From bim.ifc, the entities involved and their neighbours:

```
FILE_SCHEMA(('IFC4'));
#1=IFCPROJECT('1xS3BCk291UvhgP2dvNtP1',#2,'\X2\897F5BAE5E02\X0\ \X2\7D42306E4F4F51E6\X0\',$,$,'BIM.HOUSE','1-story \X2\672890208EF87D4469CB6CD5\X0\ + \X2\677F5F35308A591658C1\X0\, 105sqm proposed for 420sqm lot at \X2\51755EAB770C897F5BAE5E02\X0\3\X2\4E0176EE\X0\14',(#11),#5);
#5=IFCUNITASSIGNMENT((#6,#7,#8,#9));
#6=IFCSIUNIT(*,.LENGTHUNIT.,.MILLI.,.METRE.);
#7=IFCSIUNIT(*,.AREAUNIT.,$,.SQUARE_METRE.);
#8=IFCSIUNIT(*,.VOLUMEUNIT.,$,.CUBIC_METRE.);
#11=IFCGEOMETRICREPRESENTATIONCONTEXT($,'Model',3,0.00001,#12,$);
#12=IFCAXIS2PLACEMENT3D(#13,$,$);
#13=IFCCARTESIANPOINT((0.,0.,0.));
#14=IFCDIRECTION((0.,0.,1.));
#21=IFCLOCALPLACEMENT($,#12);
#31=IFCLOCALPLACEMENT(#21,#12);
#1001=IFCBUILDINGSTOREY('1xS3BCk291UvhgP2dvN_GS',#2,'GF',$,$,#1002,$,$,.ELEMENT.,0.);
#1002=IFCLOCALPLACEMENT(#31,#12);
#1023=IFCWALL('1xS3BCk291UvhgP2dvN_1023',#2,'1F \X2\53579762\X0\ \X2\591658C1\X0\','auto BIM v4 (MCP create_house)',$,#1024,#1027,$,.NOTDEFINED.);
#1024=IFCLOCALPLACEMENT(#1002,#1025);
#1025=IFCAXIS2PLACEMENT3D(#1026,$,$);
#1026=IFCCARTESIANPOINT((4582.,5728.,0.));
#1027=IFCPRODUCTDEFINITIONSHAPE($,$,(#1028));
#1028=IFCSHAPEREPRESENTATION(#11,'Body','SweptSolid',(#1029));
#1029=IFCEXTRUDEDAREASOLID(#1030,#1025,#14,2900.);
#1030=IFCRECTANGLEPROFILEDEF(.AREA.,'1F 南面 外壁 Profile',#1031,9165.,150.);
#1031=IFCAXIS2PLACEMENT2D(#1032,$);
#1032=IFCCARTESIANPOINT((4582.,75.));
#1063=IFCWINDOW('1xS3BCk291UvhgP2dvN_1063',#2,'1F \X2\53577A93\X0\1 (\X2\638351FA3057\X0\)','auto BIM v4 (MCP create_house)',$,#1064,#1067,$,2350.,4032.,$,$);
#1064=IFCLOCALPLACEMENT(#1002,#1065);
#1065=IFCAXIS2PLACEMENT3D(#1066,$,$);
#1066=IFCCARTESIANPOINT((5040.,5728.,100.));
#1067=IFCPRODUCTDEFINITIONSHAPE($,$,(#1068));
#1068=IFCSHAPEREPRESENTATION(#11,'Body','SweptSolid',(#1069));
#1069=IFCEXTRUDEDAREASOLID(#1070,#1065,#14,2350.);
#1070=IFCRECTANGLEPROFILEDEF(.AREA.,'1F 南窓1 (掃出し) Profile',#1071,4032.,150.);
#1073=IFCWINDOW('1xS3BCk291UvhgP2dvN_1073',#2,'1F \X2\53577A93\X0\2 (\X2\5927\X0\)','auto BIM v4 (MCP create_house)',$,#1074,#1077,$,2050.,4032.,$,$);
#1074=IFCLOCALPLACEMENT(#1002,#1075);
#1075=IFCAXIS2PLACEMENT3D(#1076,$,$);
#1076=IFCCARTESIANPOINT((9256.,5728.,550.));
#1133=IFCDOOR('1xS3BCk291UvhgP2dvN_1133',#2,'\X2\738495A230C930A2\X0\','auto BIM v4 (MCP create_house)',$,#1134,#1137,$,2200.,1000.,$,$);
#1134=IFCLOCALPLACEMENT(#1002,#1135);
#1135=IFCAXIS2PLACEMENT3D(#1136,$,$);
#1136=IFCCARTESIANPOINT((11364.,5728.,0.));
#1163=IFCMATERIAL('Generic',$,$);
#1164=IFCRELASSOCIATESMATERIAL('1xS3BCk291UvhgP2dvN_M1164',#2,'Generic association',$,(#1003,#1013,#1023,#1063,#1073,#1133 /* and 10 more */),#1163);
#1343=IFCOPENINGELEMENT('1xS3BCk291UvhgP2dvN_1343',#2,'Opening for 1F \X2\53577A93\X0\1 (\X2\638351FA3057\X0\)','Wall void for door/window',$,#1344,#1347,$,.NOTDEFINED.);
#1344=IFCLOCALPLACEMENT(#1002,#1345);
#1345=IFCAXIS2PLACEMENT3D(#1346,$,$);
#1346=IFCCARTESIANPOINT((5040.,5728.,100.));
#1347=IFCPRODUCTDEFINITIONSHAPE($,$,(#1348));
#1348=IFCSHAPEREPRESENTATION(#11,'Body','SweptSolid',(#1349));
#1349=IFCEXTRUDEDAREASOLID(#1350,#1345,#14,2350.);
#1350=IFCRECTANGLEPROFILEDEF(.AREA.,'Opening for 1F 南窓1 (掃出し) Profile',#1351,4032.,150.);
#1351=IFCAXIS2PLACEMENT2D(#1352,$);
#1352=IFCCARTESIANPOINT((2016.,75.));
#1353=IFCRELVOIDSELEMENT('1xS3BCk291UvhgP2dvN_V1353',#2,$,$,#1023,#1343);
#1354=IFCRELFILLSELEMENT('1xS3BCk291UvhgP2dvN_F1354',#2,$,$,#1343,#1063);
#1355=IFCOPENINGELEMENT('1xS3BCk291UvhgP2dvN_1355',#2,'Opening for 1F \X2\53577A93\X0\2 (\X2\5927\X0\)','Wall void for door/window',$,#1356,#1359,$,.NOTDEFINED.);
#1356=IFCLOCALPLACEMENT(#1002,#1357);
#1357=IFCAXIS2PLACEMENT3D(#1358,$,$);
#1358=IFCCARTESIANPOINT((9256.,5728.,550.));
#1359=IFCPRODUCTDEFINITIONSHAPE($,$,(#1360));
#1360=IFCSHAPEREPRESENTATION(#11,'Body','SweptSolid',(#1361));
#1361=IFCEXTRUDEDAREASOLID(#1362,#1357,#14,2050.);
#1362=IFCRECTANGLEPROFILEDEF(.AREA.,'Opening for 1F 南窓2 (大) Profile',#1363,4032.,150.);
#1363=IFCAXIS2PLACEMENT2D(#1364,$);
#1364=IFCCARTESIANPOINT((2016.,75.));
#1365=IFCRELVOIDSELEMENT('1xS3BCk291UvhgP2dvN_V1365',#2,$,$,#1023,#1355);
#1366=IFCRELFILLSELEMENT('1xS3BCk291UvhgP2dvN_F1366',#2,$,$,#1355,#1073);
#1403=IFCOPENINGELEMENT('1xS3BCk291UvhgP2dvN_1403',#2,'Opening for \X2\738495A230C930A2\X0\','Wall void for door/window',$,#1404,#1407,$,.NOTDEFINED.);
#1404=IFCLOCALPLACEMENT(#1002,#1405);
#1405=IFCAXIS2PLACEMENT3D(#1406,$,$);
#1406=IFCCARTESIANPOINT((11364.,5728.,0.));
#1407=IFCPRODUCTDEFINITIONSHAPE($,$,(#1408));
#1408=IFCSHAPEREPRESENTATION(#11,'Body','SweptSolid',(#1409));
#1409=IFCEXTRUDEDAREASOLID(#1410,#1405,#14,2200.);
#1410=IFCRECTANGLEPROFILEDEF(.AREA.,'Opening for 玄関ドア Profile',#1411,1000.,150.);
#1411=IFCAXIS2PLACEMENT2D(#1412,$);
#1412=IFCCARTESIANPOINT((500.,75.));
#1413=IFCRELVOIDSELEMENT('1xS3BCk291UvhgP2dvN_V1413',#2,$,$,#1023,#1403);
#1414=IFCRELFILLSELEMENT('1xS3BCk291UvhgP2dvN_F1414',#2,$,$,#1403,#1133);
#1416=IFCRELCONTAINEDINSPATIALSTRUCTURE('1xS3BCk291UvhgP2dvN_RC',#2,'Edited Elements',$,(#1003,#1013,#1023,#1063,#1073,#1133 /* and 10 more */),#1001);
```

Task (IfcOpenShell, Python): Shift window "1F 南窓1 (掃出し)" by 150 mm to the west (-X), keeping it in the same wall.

```python
import ifcopenshell
import ifcopenshell.api.geometry
import ifcopenshell.util.placement
import ifcopenshell.util.unit

model = ifcopenshell.open("bim.ifc")
unit_scale = ifcopenshell.util.unit.calculate_unit_scale(model)

window = model.by_guid("1xS3BCk291UvhgP2dvN_1063")
opening = window.FillsVoids[0].RelatingOpeningElement
wall = opening.VoidsElements[0].RelatingBuildingElement

wall_matrix = ifcopenshell.util.placement.get_local_placement(wall.ObjectPlacement)
shift = wall_matrix[:3, 0] * -0.15 / unit_scale
before = ifcopenshell.util.placement.get_local_placement(window.ObjectPlacement)[:3, 3].copy()

# The window is not placed relative to its opening, so move both.
for product in (opening, window):
    matrix = ifcopenshell.util.placement.get_local_placement(product.ObjectPlacement)
    matrix[:3, 3] += shift
    ifcopenshell.api.geometry.edit_object_placement(model, product=product, matrix=matrix, is_si=False)

after = ifcopenshell.util.placement.get_local_placement(window.ObjectPlacement)[:3, 3]
print("window moved by", (after - before).round(3) + 0.0)

model.write("bim_updated.ifc")
```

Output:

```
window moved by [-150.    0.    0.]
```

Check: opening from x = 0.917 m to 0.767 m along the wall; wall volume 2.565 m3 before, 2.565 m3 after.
